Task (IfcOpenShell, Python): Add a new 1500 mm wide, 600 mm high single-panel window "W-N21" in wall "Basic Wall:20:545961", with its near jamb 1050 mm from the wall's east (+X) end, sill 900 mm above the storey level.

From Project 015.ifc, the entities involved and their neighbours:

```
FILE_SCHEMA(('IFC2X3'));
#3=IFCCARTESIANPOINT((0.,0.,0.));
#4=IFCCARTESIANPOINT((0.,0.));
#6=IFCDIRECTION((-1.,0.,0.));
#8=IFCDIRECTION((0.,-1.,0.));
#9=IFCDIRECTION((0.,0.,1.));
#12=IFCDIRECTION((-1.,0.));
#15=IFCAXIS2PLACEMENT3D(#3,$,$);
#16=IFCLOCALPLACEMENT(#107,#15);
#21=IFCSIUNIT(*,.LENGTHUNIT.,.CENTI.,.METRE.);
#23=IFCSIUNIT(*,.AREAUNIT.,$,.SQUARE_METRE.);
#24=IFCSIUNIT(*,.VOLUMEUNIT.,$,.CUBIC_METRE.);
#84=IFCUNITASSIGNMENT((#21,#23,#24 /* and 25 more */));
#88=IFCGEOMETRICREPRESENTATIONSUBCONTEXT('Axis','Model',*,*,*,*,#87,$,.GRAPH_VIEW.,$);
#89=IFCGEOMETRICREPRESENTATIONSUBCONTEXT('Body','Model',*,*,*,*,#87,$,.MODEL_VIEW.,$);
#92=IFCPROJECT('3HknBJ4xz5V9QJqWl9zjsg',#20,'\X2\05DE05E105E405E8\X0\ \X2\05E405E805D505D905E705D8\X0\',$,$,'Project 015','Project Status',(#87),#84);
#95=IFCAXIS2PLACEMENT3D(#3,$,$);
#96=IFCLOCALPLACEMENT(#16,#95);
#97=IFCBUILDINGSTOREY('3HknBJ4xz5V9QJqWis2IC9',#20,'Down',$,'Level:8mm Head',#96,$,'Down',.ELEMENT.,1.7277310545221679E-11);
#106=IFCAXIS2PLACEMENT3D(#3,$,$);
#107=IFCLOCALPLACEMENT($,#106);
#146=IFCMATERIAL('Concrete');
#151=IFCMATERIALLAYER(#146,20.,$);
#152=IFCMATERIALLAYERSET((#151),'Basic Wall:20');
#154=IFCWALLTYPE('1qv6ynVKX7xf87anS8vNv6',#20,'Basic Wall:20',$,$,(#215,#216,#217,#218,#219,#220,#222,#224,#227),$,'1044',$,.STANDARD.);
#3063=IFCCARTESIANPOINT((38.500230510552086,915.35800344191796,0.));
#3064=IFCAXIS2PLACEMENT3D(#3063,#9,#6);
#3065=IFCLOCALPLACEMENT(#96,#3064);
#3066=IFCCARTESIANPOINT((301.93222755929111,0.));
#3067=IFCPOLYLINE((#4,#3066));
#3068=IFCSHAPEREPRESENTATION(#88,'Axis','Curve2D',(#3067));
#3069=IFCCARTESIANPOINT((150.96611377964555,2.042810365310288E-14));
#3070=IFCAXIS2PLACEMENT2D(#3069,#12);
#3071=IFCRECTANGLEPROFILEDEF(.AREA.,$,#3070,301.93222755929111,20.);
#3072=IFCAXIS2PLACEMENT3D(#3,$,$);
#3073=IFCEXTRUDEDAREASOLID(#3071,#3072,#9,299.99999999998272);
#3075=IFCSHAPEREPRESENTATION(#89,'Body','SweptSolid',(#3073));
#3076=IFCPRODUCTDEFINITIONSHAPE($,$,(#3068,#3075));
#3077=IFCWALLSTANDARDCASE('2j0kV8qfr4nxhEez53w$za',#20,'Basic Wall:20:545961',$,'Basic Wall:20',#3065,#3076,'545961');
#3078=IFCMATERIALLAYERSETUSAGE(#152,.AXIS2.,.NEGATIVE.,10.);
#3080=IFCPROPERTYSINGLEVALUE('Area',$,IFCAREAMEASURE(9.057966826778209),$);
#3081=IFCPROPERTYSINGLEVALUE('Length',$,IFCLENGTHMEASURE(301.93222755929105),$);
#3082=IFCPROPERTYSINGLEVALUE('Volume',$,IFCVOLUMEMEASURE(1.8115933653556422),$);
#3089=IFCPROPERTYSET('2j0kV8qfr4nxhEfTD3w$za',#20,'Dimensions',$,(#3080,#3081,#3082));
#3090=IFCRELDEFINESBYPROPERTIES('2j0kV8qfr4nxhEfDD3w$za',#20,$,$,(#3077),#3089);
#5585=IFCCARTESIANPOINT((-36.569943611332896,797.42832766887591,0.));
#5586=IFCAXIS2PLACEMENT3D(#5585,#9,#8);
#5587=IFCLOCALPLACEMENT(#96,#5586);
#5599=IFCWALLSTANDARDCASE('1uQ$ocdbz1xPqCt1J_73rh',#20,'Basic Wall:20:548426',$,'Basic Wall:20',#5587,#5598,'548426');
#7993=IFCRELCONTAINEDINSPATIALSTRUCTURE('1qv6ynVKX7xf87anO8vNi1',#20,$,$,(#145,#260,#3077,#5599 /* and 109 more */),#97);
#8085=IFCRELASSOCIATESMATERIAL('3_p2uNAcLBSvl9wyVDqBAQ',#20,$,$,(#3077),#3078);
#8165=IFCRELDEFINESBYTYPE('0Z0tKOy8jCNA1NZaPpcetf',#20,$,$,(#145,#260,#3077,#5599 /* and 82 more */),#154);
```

```python
import numpy as np
import ifcopenshell
import ifcopenshell.api.feature
import ifcopenshell.api.geometry
import ifcopenshell.api.pset
import ifcopenshell.api.root
import ifcopenshell.api.spatial
import ifcopenshell.api.type
import ifcopenshell.geom
import ifcopenshell.util.element
import ifcopenshell.util.placement
import ifcopenshell.util.representation
import ifcopenshell.util.shape
import ifcopenshell.util.unit

model = ifcopenshell.open("Project 015.ifc")
unit_scale = ifcopenshell.util.unit.calculate_unit_scale(model)
area_scale = ifcopenshell.util.unit.calculate_unit_scale(model, "AREAUNIT")
volume_scale = ifcopenshell.util.unit.calculate_unit_scale(model, "VOLUMEUNIT")
settings = ifcopenshell.geom.settings()


def volume(element):
    """Net volume in cubic metres, openings subtracted."""
    shape = ifcopenshell.geom.create_shape(settings, element)
    return ifcopenshell.util.shape.get_volume(shape.geometry)


wall = model.by_guid("2j0kV8qfr4nxhEez53w$za")
storey = ifcopenshell.util.element.get_container(wall, ifc_class="IfcBuildingStorey")
context = ifcopenshell.util.representation.get_context(model, "Model", "Body", "MODEL_VIEW")
before = volume(wall)

width, height, from_end, sill = 1.5, 0.6, 1.05, 0.9  # metres

# The wall runs along its own X axis, and the end named is its -X end.
wall_shape = ifcopenshell.geom.create_shape(settings, wall)
x, y, z = ifcopenshell.util.shape.get_vertices(wall_shape.geometry).T
start = x.min() + from_end
face, thickness = float(y.min()), float(y.max() - y.min())
wall_matrix = ifcopenshell.util.placement.get_local_placement(wall.ObjectPlacement)
level = ifcopenshell.util.placement.get_local_placement(storey.ObjectPlacement)[2, 3]


def in_wall(x, y):
    """Placement at x, y metres in the wall's axes, at sill height."""
    matrix = wall_matrix.copy()
    matrix[:, 3] = wall_matrix @ np.array([x / unit_scale, y / unit_scale, 0.0, 1.0])
    matrix[2, 3] = level + sill / unit_scale
    return matrix


# Opening: a box that overshoots both wall faces by 50 mm.
opening = ifcopenshell.api.root.create_entity(model, ifc_class="IfcOpeningElement")
box = ifcopenshell.api.geometry.add_wall_representation(
    model, context=context, length=width, height=height, thickness=thickness + 0.1
)
ifcopenshell.api.geometry.assign_representation(model, product=opening, representation=box)
ifcopenshell.api.geometry.edit_object_placement(model, product=opening, matrix=in_wall(start, face - 0.05), is_si=False)
ifcopenshell.api.feature.add_feature(model, feature=opening, element=wall)

window = ifcopenshell.api.root.create_entity(model, ifc_class="IfcWindow", name="W-N21")
window.OverallWidth, window.OverallHeight = width / unit_scale, height / unit_scale
body = ifcopenshell.api.geometry.add_window_representation(
    model,
    context=context,
    overall_width=window.OverallWidth,
    overall_height=window.OverallHeight,
    partition_type="SINGLE_PANEL",
)
ifcopenshell.api.geometry.assign_representation(model, product=window, representation=body)
ifcopenshell.api.spatial.assign_container(model, products=[window], relating_structure=storey)
fills = ifcopenshell.api.feature.add_filling(model, opening=opening, element=window)
fills.OwnerHistory = window.OwnerHistory  # required in IFC2X3

# IFC2X3 keeps the operation on the window style.
style = ifcopenshell.api.root.create_entity(model, ifc_class="IfcWindowStyle", name="W-N21")
style.OperationType, style.ConstructionType = "SINGLE_PANEL", "NOTDEFINED"
style.ParameterTakesPrecedence = style.Sizeable = False
ifcopenshell.api.type.assign_type(model, related_objects=[window], relating_type=style)

# Centre the window in the wall's thickness.
ifcopenshell.api.geometry.edit_object_placement(model, product=window, matrix=in_wall(start, face), is_si=False)
window_shape = ifcopenshell.geom.create_shape(settings, window)
depth = ifcopenshell.util.shape.get_vertices(window_shape.geometry)[:, 1]
offset = face + thickness / 2 - (depth.min() + depth.max()) / 2
ifcopenshell.api.geometry.edit_object_placement(model, product=window, matrix=in_wall(start, offset), is_si=False)

after = volume(wall)

# Update the wall's stored quantities.
pset = model.by_id(ifcopenshell.util.element.get_pset(wall, "Dimensions", should_inherit=False)["id"])
ifcopenshell.api.pset.edit_pset(model, pset=pset, properties={
    "Area": model.create_entity("IfcAreaMeasure", after / thickness / area_scale),
    "Volume": model.create_entity("IfcVolumeMeasure", after / volume_scale),
})

print(f"wall volume {before:.3f} -> {after:.3f} m3")

model.write("Project 015-out.ifc")
```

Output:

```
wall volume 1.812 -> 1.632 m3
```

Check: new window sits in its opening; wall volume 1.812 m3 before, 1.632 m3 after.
